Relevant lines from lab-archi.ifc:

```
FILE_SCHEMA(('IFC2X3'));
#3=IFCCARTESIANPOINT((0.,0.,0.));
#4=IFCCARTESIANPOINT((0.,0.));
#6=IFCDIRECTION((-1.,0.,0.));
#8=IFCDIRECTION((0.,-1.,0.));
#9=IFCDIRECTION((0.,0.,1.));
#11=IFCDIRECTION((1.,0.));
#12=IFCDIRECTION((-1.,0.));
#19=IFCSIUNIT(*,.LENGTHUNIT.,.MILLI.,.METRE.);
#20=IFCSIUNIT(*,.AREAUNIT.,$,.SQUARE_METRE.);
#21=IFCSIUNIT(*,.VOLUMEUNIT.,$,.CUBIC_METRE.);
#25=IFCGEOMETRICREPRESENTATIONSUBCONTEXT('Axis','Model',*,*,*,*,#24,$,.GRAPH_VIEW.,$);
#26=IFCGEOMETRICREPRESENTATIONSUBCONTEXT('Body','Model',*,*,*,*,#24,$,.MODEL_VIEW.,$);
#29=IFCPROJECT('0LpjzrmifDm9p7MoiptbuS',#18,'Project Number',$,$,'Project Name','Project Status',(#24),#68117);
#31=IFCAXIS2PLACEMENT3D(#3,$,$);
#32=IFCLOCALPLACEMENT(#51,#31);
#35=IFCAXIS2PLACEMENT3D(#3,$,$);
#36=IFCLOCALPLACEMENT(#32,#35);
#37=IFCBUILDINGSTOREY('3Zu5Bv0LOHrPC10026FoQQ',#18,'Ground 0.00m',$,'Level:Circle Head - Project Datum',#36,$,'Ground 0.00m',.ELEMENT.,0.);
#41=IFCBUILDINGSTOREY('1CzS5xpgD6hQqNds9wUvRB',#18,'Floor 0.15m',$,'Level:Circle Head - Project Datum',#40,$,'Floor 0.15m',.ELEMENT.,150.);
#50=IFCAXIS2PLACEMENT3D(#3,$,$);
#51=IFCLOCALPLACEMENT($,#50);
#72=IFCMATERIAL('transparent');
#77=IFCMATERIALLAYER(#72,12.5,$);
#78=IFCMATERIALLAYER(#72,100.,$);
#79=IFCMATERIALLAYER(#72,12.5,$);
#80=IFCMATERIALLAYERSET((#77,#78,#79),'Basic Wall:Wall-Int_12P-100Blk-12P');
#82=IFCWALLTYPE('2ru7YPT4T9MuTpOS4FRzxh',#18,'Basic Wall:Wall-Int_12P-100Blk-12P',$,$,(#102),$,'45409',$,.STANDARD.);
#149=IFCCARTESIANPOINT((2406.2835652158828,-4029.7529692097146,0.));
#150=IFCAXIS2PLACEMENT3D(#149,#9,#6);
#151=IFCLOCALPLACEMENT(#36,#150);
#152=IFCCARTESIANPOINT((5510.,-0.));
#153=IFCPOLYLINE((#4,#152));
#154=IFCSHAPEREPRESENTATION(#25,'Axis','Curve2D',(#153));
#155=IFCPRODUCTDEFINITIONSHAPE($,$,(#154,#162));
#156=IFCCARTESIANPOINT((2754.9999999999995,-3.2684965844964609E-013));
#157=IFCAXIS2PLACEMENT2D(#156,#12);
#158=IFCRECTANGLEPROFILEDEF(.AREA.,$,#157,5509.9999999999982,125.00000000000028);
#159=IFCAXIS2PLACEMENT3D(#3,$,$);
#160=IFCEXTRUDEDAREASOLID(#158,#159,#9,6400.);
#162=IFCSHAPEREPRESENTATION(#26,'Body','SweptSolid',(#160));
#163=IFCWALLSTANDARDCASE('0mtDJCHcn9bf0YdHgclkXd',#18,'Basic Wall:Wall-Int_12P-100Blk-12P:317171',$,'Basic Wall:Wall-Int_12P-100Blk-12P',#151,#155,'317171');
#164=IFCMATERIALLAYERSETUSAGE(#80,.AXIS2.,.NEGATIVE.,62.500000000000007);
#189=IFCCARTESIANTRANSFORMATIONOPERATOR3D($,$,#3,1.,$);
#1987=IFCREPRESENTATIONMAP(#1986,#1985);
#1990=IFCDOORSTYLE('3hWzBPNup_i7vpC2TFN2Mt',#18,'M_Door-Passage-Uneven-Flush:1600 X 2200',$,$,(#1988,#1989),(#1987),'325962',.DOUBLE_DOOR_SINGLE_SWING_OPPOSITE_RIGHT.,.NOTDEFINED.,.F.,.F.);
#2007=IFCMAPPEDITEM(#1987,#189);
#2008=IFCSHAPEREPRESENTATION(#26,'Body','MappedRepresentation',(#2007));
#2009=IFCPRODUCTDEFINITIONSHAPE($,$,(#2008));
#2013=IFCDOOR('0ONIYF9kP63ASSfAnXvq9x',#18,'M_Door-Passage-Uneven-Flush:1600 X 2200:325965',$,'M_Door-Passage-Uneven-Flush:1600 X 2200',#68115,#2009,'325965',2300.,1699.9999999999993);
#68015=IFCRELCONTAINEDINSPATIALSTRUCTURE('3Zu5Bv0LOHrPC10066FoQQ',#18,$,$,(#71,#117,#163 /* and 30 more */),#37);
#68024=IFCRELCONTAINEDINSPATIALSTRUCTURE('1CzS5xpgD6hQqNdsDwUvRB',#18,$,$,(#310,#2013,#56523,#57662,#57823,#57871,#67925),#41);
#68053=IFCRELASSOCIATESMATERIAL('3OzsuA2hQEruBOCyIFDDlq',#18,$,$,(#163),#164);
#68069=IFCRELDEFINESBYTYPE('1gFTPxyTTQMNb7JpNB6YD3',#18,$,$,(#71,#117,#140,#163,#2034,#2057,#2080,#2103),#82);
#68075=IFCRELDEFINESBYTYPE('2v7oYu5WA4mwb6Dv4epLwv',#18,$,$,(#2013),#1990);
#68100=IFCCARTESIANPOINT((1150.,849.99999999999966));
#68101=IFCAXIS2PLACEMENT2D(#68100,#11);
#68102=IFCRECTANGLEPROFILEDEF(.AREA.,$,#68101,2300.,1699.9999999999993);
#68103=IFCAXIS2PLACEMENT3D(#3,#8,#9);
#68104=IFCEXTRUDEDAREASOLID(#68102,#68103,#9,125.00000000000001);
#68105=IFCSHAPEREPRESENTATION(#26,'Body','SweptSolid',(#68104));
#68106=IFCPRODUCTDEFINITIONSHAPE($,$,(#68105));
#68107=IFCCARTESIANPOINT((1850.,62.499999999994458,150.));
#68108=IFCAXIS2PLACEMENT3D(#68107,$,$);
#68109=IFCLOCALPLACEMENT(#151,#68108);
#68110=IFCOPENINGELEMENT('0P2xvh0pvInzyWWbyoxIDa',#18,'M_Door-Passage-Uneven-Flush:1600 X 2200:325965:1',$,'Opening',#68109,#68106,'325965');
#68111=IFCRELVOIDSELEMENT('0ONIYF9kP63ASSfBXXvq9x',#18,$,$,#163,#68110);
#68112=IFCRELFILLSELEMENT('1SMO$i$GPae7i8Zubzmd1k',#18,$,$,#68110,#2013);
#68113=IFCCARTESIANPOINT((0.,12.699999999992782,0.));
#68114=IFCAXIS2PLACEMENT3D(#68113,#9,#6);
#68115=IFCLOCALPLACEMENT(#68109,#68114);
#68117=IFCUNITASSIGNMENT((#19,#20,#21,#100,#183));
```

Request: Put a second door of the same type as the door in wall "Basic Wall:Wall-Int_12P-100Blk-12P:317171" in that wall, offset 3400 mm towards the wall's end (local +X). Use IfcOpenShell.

```python
import ifcopenshell
import ifcopenshell.api.feature
import ifcopenshell.api.geometry
import ifcopenshell.api.root
import ifcopenshell.geom
import ifcopenshell.util.element
import ifcopenshell.util.placement
import ifcopenshell.util.shape

model = ifcopenshell.open("lab-archi.ifc")
settings = ifcopenshell.geom.settings()


def volume(element):
    """Net volume in cubic metres, openings subtracted."""
    shape = ifcopenshell.geom.create_shape(settings, element)
    return ifcopenshell.util.shape.get_volume(shape.geometry)


def reuse_history(source, copy):
    """copy_class also copies each property set's owner history, people and application; keep the originals."""
    for rel in copy.IsDefinedBy:
        if rel.is_a("IfcRelDefinesByProperties") and (history := rel.RelatingPropertyDefinition.OwnerHistory):
            rel.RelatingPropertyDefinition.OwnerHistory = source.OwnerHistory
            ifcopenshell.util.element.remove_deep2(model, history)


door = model.by_guid("0ONIYF9kP63ASSfAnXvq9x")
opening = door.FillsVoids[0].RelatingOpeningElement
wall = opening.VoidsElements[0].RelatingBuildingElement
before = volume(wall)
shift = ifcopenshell.util.placement.get_local_placement(wall.ObjectPlacement)[:3, 0] * 3400.0

# copy_class copies the void relationship, type, container and properties, but no geometry.
new_opening = ifcopenshell.api.root.copy_class(model, product=opening)
new_opening.Representation = ifcopenshell.util.element.copy_deep(
    model, opening.Representation, exclude=["IfcGeometricRepresentationContext", "IfcRepresentationMap"]
)
new_opening.Name = "M_Door-Passage-Uneven-Flush:1600 X 2200"
new_opening.Tag = None
new_door = ifcopenshell.api.root.copy_class(model, product=door)
new_door.Representation = ifcopenshell.util.element.copy_deep(
    model, door.Representation, exclude=["IfcGeometricRepresentationContext", "IfcRepresentationMap"]
)
new_door.Name = "M_Door-Passage-Uneven-Flush:1600 X 2200"
new_door.Tag = None
reuse_history(door, new_door)
fills = ifcopenshell.api.feature.add_filling(model, opening=new_opening, element=new_door)
fills.OwnerHistory = new_door.OwnerHistory  # required in IFC2X3

for old, new in ((opening, new_opening), (door, new_door)):
    matrix = ifcopenshell.util.placement.get_local_placement(old.ObjectPlacement)
    matrix[:3, 3] += shift
    ifcopenshell.api.geometry.edit_object_placement(model, product=new, matrix=matrix, is_si=False)

after = volume(wall)

print(f"wall volume {before:.3f} -> {after:.3f} m3")

model.write("lab-archi_edited.ifc")
```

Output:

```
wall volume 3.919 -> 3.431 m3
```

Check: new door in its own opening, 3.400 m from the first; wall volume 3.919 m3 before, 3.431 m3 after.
